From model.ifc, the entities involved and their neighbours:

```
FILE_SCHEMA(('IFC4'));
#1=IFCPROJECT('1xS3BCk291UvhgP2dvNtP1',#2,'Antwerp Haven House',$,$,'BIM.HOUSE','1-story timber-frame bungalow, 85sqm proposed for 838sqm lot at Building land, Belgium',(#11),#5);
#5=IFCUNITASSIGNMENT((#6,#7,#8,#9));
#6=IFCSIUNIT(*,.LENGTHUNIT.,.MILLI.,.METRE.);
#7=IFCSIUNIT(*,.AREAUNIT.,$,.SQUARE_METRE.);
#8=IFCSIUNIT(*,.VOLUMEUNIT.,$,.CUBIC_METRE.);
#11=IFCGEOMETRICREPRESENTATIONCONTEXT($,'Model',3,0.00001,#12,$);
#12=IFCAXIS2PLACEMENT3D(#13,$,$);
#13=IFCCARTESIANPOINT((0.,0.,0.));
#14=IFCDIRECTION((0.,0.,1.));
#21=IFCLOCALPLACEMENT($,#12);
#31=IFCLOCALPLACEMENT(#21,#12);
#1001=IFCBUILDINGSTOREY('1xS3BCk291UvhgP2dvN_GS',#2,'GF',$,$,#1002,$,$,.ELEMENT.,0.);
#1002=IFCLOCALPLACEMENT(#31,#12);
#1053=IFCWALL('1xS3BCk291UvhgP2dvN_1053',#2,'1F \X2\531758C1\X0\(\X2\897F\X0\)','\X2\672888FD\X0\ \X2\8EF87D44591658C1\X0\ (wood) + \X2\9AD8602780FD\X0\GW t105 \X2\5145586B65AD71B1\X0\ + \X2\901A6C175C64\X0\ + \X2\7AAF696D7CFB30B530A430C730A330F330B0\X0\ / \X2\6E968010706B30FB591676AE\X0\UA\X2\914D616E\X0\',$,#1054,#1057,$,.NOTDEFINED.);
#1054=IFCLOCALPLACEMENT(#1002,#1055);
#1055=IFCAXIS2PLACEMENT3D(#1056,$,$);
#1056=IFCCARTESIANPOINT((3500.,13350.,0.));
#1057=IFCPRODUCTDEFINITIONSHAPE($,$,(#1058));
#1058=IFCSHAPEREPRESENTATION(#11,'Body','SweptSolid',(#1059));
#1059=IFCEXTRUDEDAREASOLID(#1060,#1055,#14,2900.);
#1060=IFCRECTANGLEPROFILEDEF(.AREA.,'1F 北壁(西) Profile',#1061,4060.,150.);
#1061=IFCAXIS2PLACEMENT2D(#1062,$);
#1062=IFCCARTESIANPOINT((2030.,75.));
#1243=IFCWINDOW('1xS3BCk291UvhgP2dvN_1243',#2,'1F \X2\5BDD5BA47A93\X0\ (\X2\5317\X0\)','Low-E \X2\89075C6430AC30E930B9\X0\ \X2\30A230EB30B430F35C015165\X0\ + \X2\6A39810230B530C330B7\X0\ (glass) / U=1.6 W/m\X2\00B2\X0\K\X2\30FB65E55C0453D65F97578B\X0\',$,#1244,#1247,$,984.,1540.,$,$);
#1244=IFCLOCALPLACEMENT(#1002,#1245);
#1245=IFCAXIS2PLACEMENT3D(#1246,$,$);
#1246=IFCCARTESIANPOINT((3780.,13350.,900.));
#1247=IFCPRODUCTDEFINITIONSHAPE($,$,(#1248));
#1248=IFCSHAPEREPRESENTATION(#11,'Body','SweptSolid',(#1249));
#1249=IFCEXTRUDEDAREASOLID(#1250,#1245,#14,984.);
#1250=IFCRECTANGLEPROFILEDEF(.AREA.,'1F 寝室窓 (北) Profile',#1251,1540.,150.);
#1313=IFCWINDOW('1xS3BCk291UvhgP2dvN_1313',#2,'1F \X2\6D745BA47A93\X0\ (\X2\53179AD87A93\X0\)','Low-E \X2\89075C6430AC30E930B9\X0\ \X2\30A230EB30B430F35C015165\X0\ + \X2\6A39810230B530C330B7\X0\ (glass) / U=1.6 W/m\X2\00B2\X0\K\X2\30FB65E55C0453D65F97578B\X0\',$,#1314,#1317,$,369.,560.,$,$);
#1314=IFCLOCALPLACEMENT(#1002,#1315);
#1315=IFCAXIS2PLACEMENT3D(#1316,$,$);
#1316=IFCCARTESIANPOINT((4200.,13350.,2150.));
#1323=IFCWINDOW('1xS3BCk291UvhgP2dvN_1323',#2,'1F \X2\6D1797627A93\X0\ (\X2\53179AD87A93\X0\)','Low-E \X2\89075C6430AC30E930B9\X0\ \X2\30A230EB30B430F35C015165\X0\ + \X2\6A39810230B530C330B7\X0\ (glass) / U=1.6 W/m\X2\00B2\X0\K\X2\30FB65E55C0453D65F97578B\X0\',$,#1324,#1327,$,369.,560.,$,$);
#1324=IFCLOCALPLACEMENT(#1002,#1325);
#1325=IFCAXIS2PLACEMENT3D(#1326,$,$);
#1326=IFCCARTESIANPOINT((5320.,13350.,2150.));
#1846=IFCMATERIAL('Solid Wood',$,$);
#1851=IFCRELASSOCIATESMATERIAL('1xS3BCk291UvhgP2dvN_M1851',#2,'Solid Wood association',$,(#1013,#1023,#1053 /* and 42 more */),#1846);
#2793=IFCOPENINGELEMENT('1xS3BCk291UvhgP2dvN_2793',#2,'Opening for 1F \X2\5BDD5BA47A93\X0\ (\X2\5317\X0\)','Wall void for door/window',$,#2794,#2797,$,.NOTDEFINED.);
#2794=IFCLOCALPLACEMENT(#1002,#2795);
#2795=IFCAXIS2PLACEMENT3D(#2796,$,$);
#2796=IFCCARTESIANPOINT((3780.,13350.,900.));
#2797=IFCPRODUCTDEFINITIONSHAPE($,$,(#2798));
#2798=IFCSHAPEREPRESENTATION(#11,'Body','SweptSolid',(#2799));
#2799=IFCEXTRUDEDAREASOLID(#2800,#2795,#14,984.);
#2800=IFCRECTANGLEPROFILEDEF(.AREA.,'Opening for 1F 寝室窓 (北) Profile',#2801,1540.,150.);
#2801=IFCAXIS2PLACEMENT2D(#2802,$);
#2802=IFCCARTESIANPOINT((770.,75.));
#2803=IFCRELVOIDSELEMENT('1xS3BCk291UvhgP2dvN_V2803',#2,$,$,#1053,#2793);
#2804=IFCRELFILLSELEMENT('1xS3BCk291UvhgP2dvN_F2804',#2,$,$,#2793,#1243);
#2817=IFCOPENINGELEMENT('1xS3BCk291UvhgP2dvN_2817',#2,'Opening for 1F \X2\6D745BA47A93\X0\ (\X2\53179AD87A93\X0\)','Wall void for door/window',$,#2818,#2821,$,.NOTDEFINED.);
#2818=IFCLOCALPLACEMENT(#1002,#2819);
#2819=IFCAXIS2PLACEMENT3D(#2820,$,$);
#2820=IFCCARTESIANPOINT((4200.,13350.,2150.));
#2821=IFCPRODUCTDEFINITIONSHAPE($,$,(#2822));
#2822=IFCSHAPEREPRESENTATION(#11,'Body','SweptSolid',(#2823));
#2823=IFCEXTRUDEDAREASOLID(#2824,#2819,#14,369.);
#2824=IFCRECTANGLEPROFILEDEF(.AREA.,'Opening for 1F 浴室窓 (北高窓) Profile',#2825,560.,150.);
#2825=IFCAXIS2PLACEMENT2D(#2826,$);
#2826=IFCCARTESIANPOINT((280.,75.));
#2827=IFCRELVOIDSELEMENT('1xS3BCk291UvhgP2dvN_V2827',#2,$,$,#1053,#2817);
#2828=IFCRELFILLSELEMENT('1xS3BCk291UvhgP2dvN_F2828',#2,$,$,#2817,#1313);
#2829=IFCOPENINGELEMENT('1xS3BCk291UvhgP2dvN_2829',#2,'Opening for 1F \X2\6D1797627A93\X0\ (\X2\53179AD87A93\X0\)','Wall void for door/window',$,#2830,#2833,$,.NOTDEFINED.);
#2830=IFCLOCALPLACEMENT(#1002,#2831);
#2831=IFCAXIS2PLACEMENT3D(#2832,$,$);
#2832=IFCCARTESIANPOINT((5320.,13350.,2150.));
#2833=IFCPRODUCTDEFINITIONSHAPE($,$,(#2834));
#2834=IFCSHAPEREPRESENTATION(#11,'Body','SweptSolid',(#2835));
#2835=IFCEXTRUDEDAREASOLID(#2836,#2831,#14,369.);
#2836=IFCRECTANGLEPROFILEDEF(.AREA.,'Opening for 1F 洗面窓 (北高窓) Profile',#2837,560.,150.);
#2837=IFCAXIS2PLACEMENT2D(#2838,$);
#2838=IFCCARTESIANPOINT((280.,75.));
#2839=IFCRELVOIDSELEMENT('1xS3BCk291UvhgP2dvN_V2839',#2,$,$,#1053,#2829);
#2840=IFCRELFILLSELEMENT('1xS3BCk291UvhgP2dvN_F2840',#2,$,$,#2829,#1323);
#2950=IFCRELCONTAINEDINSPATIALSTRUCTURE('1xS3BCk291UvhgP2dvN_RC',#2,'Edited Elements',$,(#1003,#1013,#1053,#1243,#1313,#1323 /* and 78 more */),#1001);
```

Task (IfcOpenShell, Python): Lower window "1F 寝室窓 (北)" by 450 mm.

```python
import numpy as np
import ifcopenshell
import ifcopenshell.api.geometry
import ifcopenshell.util.placement
import ifcopenshell.util.unit

model = ifcopenshell.open("model.ifc")
unit_scale = ifcopenshell.util.unit.calculate_unit_scale(model)

window = model.by_id(1243)
opening = window.FillsVoids[0].RelatingOpeningElement
dz = -450.0

shift = np.array([0.0, 0.0, dz])
# The window is not placed relative to its opening, so move both.
for product in (opening, window):
    matrix = ifcopenshell.util.placement.get_local_placement(product.ObjectPlacement)
    matrix[:3, 3] += shift
    ifcopenshell.api.geometry.edit_object_placement(model, product=product, matrix=matrix, is_si=False)

print(f"moved by {dz * unit_scale:+.3f} m")

model.write("model_rev.ifc")
```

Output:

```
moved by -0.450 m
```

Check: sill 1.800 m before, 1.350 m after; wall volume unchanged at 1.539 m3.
